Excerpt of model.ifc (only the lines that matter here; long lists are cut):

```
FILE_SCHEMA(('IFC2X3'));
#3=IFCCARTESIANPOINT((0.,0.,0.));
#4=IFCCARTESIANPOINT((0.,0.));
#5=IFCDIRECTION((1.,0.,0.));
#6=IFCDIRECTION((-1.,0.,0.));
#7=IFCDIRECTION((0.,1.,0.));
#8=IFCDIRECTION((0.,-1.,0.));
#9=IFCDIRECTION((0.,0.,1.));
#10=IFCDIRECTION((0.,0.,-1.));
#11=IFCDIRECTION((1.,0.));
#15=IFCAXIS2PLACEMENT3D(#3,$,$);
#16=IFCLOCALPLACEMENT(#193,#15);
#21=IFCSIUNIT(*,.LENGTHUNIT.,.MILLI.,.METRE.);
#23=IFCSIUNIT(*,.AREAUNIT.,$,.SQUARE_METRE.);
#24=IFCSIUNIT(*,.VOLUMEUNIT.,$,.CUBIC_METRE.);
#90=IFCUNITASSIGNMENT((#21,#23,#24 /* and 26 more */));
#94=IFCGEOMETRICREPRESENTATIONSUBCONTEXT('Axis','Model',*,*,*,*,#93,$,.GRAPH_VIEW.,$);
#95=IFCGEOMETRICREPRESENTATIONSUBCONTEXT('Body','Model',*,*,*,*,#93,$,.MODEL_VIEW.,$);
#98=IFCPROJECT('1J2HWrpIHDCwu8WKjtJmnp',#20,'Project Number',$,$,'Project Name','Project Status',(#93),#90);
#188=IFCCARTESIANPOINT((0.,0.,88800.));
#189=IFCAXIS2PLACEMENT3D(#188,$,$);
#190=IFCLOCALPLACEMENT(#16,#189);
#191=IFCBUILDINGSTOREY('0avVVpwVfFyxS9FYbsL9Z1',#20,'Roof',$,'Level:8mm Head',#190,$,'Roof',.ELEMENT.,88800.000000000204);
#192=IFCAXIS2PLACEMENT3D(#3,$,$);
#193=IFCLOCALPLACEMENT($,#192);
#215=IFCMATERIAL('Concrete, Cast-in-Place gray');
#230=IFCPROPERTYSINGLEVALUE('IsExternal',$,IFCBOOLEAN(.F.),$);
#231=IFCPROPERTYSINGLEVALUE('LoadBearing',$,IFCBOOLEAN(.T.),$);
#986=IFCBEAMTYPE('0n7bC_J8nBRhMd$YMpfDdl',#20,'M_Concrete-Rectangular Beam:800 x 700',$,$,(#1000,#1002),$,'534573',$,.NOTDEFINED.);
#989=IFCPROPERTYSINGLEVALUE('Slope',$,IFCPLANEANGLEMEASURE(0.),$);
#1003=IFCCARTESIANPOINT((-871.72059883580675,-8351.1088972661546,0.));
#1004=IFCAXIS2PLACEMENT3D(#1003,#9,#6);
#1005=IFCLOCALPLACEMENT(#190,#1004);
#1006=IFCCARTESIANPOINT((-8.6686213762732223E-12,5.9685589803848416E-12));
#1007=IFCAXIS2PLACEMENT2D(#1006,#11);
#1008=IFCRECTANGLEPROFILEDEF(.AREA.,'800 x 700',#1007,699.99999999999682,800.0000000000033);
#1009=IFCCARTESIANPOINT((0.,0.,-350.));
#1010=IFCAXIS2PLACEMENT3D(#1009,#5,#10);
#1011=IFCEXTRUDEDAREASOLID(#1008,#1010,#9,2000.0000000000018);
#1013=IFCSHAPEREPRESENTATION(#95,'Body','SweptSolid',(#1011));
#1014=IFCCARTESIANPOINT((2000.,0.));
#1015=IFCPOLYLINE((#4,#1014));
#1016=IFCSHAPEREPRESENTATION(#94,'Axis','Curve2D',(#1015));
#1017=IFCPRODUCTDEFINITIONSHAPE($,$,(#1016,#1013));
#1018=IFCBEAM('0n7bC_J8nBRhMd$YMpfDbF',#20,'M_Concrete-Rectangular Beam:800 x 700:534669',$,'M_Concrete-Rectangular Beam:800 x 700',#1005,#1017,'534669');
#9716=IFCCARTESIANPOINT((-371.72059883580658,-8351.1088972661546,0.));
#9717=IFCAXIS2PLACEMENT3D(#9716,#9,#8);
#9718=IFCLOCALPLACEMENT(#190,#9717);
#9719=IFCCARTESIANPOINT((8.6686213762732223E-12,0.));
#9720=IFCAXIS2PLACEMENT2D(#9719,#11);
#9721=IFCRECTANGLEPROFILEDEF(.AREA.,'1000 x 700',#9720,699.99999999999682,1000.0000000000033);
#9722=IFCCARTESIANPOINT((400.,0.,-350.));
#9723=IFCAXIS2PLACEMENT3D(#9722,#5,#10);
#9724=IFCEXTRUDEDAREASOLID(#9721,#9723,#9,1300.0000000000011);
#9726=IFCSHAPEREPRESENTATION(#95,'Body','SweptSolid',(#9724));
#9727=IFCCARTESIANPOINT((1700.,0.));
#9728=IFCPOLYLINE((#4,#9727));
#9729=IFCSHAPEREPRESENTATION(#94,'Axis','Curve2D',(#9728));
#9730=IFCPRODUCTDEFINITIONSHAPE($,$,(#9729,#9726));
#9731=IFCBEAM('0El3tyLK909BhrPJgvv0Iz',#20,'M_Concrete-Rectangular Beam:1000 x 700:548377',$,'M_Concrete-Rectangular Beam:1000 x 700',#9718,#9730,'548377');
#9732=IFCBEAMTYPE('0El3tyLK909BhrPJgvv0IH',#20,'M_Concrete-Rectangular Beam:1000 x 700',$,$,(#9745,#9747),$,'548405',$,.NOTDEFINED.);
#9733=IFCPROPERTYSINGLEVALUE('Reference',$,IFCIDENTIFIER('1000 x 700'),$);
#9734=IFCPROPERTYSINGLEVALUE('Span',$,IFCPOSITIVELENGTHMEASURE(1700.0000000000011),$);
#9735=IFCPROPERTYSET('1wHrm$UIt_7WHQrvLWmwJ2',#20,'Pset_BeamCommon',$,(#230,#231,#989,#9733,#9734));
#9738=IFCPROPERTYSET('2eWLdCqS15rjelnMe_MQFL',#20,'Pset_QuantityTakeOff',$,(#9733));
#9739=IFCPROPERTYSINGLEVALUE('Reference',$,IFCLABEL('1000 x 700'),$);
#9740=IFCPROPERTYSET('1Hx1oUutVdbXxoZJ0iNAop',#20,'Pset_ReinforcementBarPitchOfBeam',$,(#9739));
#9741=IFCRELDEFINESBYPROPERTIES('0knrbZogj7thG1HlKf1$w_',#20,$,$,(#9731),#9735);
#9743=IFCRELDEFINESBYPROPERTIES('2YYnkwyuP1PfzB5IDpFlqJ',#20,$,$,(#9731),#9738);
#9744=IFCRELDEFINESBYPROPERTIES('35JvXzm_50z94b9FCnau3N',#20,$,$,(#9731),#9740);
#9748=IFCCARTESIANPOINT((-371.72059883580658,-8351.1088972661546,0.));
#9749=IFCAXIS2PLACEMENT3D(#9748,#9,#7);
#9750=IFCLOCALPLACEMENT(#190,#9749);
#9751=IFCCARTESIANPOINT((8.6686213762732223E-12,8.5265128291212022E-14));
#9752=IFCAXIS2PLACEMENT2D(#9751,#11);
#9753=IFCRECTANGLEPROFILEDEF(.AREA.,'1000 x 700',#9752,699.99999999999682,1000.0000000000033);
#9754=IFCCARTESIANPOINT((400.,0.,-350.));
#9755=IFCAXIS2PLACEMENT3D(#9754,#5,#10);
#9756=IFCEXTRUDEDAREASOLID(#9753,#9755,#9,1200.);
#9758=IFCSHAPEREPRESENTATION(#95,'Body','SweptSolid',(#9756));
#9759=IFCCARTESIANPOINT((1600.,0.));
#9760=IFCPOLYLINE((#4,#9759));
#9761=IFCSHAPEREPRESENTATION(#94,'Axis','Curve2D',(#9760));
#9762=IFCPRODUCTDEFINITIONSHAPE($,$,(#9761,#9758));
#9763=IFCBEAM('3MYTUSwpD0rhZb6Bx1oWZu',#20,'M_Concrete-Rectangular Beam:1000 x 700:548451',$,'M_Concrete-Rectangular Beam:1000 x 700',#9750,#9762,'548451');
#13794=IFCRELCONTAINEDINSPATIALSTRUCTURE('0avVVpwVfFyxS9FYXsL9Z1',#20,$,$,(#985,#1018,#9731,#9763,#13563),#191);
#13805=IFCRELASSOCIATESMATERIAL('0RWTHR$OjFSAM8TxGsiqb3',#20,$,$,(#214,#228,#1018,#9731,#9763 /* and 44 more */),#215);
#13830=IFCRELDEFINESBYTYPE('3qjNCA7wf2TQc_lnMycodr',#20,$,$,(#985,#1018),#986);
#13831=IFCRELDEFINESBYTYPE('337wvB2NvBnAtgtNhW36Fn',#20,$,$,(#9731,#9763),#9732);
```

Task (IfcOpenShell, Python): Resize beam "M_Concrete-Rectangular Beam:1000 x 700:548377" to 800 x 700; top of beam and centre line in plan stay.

```python
import ifcopenshell
import ifcopenshell.api.pset
import ifcopenshell.api.type
import ifcopenshell.util.element
import ifcopenshell.util.representation

model = ifcopenshell.open("model.ifc")

member = model.by_id(9731)
source = next(p for p in model.by_type("IfcRectangleProfileDef") if p.ProfileName == "800 x 700")

body = ifcopenshell.util.representation.get_representation(member, "Model", "Body")
solid = body.Items[0]
old_profile = solid.SweptArea

# Copy the section's sizes but keep this member's own profile position.
profile = ifcopenshell.util.element.copy(model, source)
# Profiles are centred, so shift by half the change in depth to hold the top.
shift = (old_profile.XDim - profile.XDim) / 2
x, y = old_profile.Position.Location.Coordinates
up = (-1.0, 0.0)  # upwards, in the solid's own plane
location = model.createIfcCartesianPoint((x + up[0] * shift, y + up[1] * shift))
profile.Position = model.createIfcAxis2Placement2D(location, old_profile.Position.RefDirection)
solid.SweptArea = profile
if not model.get_total_inverses(old_profile):
    ifcopenshell.util.element.remove_deep2(model, old_profile)

new_type = model.by_guid("0n7bC_J8nBRhMd$YMpfDdl")
ifcopenshell.api.type.assign_type(
    model, related_objects=[member], relating_type=new_type, should_map_representations=False
)
member.Name = member.Name.replace("1000 x 700", "800 x 700")
member.ObjectType = "M_Concrete-Rectangular Beam:800 x 700"
pset = model.by_id(ifcopenshell.util.element.get_pset(member, "Pset_BeamCommon", should_inherit=False)["id"])
ifcopenshell.api.pset.edit_pset(model, pset=pset, properties={"Reference": "800 x 700"})
pset = model.by_id(ifcopenshell.util.element.get_pset(member, "Pset_QuantityTakeOff", should_inherit=False)["id"])
ifcopenshell.api.pset.edit_pset(model, pset=pset, properties={"Reference": "800 x 700"})
pset = model.by_id(ifcopenshell.util.element.get_pset(member, "Pset_ReinforcementBarPitchOfBeam", should_inherit=False)["id"])
ifcopenshell.api.pset.edit_pset(model, pset=pset, properties={"Reference": "800 x 700"})

print(solid.SweptArea)

model.write("model_updated.ifc")
```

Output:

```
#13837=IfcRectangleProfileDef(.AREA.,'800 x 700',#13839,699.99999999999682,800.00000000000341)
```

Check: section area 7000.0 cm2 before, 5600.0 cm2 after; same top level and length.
